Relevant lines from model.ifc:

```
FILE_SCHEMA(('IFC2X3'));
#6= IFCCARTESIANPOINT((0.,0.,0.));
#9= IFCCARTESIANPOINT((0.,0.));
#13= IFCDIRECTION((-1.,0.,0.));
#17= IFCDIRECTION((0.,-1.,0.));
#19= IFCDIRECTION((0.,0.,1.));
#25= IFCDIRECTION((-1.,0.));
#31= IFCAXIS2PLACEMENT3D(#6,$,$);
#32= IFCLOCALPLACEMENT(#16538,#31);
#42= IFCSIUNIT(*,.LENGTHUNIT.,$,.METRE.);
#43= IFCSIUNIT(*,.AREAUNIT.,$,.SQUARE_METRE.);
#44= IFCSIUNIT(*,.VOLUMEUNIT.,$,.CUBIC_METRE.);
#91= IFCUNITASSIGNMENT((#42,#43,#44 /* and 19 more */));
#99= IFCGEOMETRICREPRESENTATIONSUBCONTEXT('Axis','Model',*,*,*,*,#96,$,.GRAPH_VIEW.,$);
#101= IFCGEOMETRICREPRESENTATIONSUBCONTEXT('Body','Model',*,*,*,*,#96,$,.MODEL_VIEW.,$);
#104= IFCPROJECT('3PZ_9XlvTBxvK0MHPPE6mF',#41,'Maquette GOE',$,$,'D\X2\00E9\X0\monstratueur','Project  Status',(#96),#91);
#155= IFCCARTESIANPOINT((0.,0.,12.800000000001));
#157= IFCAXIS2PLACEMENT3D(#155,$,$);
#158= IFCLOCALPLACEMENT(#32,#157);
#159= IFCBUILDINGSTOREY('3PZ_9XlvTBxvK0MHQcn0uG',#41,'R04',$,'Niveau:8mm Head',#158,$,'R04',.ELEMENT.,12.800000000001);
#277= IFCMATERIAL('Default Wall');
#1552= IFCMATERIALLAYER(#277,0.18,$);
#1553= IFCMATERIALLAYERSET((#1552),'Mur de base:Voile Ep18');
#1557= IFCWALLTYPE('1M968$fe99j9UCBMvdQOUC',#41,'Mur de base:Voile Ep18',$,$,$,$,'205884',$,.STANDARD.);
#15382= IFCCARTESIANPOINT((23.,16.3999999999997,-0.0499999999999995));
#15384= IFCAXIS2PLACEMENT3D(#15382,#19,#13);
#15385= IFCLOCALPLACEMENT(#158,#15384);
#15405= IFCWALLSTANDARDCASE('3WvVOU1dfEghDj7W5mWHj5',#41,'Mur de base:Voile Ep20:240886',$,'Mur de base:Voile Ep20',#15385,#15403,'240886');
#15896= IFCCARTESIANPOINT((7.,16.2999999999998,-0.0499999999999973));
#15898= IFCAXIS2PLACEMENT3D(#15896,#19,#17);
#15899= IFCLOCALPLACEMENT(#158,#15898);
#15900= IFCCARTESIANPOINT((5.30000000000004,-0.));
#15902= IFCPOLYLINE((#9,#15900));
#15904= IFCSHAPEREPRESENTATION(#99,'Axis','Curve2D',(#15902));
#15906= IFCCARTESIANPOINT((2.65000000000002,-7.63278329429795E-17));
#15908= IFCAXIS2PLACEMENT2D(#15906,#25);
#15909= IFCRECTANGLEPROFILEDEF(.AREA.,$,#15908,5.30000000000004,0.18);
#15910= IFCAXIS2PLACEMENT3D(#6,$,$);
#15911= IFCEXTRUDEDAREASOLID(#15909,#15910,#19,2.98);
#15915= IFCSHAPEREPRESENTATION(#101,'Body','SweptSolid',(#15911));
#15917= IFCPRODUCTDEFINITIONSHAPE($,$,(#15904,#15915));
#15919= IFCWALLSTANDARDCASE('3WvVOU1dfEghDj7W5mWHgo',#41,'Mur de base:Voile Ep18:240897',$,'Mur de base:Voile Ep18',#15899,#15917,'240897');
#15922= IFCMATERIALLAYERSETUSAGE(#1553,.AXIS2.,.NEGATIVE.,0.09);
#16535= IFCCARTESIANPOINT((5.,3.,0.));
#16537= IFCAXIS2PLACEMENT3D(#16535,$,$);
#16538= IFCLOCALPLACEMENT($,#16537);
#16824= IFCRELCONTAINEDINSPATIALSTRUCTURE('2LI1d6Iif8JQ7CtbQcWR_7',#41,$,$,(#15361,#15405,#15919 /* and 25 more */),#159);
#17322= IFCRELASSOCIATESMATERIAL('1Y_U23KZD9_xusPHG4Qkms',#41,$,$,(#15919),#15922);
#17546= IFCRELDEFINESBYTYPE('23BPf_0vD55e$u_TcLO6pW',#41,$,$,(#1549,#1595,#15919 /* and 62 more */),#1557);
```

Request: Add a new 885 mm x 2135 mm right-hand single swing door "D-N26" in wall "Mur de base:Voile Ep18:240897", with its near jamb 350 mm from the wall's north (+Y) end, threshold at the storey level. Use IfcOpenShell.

```python
import numpy as np
import ifcopenshell
import ifcopenshell.api.feature
import ifcopenshell.api.geometry
import ifcopenshell.api.root
import ifcopenshell.api.spatial
import ifcopenshell.api.type
import ifcopenshell.geom
import ifcopenshell.util.element
import ifcopenshell.util.placement
import ifcopenshell.util.representation
import ifcopenshell.util.shape
import ifcopenshell.util.unit

model = ifcopenshell.open("model.ifc")
unit_scale = ifcopenshell.util.unit.calculate_unit_scale(model)
settings = ifcopenshell.geom.settings()


def volume(element):
    """Net volume in cubic metres, openings subtracted."""
    shape = ifcopenshell.geom.create_shape(settings, element)
    return ifcopenshell.util.shape.get_volume(shape.geometry)


wall = model.by_guid("3WvVOU1dfEghDj7W5mWHgo")
storey = ifcopenshell.util.element.get_container(wall, ifc_class="IfcBuildingStorey")
context = ifcopenshell.util.representation.get_context(model, "Model", "Body", "MODEL_VIEW")
before = volume(wall)

width, height, from_end, sill = 0.885, 2.135, 0.35, 0.0  # metres

# The wall runs along its own X axis, and the end named is its -X end.
wall_shape = ifcopenshell.geom.create_shape(settings, wall)
x, y, z = ifcopenshell.util.shape.get_vertices(wall_shape.geometry).T
start = x.min() + from_end
face, thickness = float(y.min()), float(y.max() - y.min())
wall_matrix = ifcopenshell.util.placement.get_local_placement(wall.ObjectPlacement)
level = ifcopenshell.util.placement.get_local_placement(storey.ObjectPlacement)[2, 3]


def in_wall(x, y):
    """Placement at x, y metres in the wall's axes, at sill height."""
    matrix = wall_matrix.copy()
    matrix[:, 3] = wall_matrix @ np.array([x / unit_scale, y / unit_scale, 0.0, 1.0])
    matrix[2, 3] = level + sill / unit_scale
    return matrix


# Opening: a box that overshoots both wall faces by 50 mm.
opening = ifcopenshell.api.root.create_entity(model, ifc_class="IfcOpeningElement")
box = ifcopenshell.api.geometry.add_wall_representation(
    model, context=context, length=width, height=height, thickness=thickness + 0.1
)
ifcopenshell.api.geometry.assign_representation(model, product=opening, representation=box)
ifcopenshell.api.geometry.edit_object_placement(model, product=opening, matrix=in_wall(start, face - 0.05), is_si=False)
ifcopenshell.api.feature.add_feature(model, feature=opening, element=wall)

door = ifcopenshell.api.root.create_entity(model, ifc_class="IfcDoor", name="D-N26")
door.OverallWidth, door.OverallHeight = width / unit_scale, height / unit_scale
body = ifcopenshell.api.geometry.add_door_representation(
    model,
    context=context,
    overall_width=door.OverallWidth,
    overall_height=door.OverallHeight,
    operation_type="SINGLE_SWING_RIGHT",
    lining_properties={"LiningDepth": thickness / unit_scale, "ThresholdDepth": thickness / unit_scale},
)
ifcopenshell.api.geometry.assign_representation(model, product=door, representation=body)
ifcopenshell.api.spatial.assign_container(model, products=[door], relating_structure=storey)
fills = ifcopenshell.api.feature.add_filling(model, opening=opening, element=door)
fills.OwnerHistory = door.OwnerHistory  # required in IFC2X3

# IFC2X3 keeps the operation on the door style.
style = ifcopenshell.api.root.create_entity(model, ifc_class="IfcDoorStyle", name="D-N26")
style.OperationType, style.ConstructionType = "SINGLE_SWING_RIGHT", "NOTDEFINED"
style.ParameterTakesPrecedence = style.Sizeable = False
ifcopenshell.api.type.assign_type(model, related_objects=[door], relating_type=style)

# The lining spans the wall, so the door starts at the wall face.
ifcopenshell.api.geometry.edit_object_placement(model, product=door, matrix=in_wall(start, face), is_si=False)

after = volume(wall)

print(f"wall volume {before:.3f} -> {after:.3f} m3")

model.write("model_edited.ifc")
```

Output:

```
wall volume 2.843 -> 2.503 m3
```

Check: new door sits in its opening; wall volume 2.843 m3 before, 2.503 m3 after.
